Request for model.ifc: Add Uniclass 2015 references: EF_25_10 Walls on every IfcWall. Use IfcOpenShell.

First a look at what the model holds.

```python
import ifcopenshell

model = ifcopenshell.open("model.ifc")
print(model.schema)
print("classifications:", [c.Name for c in model.by_type("IfcClassification")])
for ifc_class in ("IfcDoor", "IfcRoof", "IfcStair", "IfcWall", "IfcWindow"):
    print(ifc_class, len(model.by_type(ifc_class)))
```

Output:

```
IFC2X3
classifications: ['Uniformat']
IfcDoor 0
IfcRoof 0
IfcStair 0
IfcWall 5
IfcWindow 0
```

```python
import ifcopenshell
import ifcopenshell.api.classification

model = ifcopenshell.open("model.ifc")

# IFC2X3 requires Source and Edition and has no link from the project to the system.
system = model.create_entity("IfcClassification", Source="NBS", Edition="2015", Name="Uniclass 2015")

codes = {
    "IfcWall": ("EF_25_10", "Walls"),
}
for ifc_class, (code, name) in codes.items():
    products = model.by_type(ifc_class)
    ifcopenshell.api.classification.add_reference(
        model, products=products, classification=system, identification=code, name=name
    )
    print(code, len(products))

model.write("model_edited.ifc")
```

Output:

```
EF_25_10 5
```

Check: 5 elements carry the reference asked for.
